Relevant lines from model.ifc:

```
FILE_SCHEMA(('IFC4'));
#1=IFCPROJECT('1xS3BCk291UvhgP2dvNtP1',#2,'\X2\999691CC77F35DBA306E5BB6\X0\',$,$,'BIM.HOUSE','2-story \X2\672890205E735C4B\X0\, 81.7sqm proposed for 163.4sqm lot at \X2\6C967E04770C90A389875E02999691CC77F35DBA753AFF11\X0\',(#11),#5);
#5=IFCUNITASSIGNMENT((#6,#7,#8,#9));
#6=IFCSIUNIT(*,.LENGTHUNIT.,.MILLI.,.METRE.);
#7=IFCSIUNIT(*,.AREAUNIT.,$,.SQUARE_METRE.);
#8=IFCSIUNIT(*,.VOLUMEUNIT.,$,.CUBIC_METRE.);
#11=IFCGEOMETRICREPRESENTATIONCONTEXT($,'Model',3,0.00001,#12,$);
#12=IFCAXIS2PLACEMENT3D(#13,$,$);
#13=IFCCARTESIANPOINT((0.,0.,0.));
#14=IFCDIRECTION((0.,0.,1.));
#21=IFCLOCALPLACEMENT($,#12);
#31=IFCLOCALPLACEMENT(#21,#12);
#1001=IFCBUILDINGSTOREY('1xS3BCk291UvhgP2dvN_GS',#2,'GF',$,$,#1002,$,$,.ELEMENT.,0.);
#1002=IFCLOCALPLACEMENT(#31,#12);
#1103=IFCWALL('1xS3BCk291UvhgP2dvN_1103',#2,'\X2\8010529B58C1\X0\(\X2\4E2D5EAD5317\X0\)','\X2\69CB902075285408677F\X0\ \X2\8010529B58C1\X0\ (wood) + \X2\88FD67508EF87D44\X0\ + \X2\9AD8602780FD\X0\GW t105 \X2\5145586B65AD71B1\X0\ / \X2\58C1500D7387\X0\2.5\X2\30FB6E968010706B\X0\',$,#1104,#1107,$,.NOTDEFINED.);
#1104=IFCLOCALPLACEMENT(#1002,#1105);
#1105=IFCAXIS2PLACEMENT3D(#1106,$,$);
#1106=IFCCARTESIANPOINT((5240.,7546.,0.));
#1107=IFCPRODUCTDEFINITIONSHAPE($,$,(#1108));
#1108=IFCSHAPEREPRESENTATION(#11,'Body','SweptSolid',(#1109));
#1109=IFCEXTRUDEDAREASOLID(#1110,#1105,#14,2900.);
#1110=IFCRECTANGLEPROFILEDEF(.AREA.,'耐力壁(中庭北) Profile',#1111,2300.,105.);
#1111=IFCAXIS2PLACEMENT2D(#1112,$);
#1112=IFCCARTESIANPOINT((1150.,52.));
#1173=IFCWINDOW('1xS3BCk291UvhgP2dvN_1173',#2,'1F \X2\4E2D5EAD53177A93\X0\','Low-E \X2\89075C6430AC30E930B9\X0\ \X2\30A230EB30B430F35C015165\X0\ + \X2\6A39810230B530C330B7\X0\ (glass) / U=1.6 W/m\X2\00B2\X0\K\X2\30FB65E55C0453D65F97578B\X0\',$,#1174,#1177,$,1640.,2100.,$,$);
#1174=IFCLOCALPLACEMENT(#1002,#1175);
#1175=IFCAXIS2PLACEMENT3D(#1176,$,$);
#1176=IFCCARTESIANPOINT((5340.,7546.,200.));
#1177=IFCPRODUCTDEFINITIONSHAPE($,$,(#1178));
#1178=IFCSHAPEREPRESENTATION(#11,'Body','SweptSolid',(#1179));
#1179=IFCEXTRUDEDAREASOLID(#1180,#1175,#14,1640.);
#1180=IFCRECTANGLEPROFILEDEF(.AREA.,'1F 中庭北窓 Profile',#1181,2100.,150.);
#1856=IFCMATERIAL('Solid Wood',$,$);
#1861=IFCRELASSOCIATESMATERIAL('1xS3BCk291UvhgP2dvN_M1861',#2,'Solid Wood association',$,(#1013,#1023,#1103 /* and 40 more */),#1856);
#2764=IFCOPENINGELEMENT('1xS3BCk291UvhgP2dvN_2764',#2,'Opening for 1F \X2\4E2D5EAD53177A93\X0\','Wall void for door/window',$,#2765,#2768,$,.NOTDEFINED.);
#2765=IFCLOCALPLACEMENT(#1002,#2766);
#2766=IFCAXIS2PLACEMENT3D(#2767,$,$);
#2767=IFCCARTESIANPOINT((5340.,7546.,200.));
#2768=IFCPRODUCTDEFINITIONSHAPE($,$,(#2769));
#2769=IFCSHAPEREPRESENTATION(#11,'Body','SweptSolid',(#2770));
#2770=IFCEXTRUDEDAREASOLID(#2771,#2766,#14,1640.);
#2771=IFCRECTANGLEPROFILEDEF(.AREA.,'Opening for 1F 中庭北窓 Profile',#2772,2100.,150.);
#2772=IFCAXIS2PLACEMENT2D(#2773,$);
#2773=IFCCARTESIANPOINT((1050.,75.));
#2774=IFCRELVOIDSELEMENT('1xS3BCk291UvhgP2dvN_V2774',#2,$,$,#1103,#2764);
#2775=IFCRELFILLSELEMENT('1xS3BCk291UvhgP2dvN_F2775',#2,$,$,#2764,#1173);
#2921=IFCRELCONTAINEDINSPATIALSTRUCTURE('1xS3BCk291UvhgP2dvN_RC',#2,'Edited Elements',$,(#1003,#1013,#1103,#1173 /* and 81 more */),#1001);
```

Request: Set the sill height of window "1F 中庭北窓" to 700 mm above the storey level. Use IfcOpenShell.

```python
import numpy as np
import ifcopenshell
import ifcopenshell.api.geometry
import ifcopenshell.geom
import ifcopenshell.util.element
import ifcopenshell.util.placement
import ifcopenshell.util.shape
import ifcopenshell.util.unit

model = ifcopenshell.open("model.ifc")
unit_scale = ifcopenshell.util.unit.calculate_unit_scale(model)

window = model.by_guid("1xS3BCk291UvhgP2dvN_1173")
opening = window.FillsVoids[0].RelatingOpeningElement
storey = ifcopenshell.util.element.get_container(window, ifc_class="IfcBuildingStorey")
level = ifcopenshell.util.placement.get_local_placement(storey.ObjectPlacement)[2, 3]

# The opening's origin need not be at the sill, so measure its lowest point.
shape = ifcopenshell.geom.create_shape(ifcopenshell.geom.settings(), opening)
bottom = ifcopenshell.util.shape.get_shape_bottom_elevation(shape, shape.geometry) / unit_scale
dz = level + 700.0 - bottom

shift = np.array([0.0, 0.0, dz])
# The window is not placed relative to its opening, so move both.
for product in (opening, window):
    matrix = ifcopenshell.util.placement.get_local_placement(product.ObjectPlacement)
    matrix[:3, 3] += shift
    ifcopenshell.api.geometry.edit_object_placement(model, product=product, matrix=matrix, is_si=False)

print(f"moved by {dz * unit_scale:+.3f} m")

model.write("model_v2.ifc")
```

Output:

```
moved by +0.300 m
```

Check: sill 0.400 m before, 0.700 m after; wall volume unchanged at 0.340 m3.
